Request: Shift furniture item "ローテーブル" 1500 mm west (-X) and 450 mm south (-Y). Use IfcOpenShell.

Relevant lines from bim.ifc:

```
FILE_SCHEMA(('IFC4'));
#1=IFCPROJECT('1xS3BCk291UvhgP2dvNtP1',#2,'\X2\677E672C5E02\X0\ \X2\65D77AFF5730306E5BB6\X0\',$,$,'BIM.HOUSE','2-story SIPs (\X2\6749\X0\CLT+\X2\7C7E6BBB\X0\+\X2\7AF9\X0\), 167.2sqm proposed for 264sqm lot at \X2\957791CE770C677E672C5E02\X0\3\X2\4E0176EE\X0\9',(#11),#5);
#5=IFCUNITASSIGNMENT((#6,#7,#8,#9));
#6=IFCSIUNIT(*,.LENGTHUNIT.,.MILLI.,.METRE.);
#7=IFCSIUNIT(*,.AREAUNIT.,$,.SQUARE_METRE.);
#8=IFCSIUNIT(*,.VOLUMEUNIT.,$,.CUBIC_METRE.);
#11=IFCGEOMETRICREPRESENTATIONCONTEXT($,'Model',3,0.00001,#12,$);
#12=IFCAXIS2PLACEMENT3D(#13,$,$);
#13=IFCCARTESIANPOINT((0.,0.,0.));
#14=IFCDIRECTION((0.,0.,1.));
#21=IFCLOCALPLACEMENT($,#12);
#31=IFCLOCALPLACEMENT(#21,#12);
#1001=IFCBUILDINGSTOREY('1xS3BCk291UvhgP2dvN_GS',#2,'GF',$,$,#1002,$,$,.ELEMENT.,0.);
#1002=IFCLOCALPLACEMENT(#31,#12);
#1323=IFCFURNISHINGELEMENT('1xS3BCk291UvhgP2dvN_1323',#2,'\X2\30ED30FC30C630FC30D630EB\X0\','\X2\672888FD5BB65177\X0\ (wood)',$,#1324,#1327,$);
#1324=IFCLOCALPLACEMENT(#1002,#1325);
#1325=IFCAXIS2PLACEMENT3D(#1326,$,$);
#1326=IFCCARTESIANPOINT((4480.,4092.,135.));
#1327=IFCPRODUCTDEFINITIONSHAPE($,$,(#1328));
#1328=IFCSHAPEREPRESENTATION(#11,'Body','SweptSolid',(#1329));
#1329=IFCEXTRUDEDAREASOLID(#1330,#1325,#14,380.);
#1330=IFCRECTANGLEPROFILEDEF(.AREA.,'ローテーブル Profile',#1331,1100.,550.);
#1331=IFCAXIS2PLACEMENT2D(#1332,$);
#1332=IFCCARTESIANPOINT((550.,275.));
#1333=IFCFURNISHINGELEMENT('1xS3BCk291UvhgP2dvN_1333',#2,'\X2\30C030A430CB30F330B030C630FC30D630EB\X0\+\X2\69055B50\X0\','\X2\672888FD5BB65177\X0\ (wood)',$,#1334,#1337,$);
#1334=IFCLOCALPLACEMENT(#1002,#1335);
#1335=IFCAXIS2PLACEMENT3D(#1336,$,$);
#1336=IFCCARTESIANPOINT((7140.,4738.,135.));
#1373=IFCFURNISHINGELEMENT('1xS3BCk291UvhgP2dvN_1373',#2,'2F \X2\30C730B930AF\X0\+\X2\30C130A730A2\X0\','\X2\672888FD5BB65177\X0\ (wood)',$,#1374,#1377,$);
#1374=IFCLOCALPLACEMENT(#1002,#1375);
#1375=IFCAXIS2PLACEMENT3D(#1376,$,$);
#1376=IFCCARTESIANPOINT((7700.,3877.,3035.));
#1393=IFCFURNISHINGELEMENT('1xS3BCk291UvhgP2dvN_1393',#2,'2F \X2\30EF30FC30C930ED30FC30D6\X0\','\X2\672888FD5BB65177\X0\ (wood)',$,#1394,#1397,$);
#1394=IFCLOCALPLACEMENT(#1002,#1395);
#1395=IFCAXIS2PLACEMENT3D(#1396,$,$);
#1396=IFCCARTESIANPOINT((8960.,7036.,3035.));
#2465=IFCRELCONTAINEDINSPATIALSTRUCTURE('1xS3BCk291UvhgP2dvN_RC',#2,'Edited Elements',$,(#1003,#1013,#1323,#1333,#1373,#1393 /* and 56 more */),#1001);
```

```python
import ifcopenshell
import ifcopenshell.api.geometry
import ifcopenshell.util.placement

model = ifcopenshell.open("bim.ifc")

item = model.by_guid("1xS3BCk291UvhgP2dvN_1323")
matrix = ifcopenshell.util.placement.get_local_placement(item.ObjectPlacement)
matrix[0, 3] -= 1500.0
matrix[1, 3] -= 450.0
ifcopenshell.api.geometry.edit_object_placement(model, product=item, matrix=matrix, is_si=False)

print(ifcopenshell.util.placement.get_local_placement(item.ObjectPlacement).round(3) + 0.0)

model.write("bim_updated.ifc")
```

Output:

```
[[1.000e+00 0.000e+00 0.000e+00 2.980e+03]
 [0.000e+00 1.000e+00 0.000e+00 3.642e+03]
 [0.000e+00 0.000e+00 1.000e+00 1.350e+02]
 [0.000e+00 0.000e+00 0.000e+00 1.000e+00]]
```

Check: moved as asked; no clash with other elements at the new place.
